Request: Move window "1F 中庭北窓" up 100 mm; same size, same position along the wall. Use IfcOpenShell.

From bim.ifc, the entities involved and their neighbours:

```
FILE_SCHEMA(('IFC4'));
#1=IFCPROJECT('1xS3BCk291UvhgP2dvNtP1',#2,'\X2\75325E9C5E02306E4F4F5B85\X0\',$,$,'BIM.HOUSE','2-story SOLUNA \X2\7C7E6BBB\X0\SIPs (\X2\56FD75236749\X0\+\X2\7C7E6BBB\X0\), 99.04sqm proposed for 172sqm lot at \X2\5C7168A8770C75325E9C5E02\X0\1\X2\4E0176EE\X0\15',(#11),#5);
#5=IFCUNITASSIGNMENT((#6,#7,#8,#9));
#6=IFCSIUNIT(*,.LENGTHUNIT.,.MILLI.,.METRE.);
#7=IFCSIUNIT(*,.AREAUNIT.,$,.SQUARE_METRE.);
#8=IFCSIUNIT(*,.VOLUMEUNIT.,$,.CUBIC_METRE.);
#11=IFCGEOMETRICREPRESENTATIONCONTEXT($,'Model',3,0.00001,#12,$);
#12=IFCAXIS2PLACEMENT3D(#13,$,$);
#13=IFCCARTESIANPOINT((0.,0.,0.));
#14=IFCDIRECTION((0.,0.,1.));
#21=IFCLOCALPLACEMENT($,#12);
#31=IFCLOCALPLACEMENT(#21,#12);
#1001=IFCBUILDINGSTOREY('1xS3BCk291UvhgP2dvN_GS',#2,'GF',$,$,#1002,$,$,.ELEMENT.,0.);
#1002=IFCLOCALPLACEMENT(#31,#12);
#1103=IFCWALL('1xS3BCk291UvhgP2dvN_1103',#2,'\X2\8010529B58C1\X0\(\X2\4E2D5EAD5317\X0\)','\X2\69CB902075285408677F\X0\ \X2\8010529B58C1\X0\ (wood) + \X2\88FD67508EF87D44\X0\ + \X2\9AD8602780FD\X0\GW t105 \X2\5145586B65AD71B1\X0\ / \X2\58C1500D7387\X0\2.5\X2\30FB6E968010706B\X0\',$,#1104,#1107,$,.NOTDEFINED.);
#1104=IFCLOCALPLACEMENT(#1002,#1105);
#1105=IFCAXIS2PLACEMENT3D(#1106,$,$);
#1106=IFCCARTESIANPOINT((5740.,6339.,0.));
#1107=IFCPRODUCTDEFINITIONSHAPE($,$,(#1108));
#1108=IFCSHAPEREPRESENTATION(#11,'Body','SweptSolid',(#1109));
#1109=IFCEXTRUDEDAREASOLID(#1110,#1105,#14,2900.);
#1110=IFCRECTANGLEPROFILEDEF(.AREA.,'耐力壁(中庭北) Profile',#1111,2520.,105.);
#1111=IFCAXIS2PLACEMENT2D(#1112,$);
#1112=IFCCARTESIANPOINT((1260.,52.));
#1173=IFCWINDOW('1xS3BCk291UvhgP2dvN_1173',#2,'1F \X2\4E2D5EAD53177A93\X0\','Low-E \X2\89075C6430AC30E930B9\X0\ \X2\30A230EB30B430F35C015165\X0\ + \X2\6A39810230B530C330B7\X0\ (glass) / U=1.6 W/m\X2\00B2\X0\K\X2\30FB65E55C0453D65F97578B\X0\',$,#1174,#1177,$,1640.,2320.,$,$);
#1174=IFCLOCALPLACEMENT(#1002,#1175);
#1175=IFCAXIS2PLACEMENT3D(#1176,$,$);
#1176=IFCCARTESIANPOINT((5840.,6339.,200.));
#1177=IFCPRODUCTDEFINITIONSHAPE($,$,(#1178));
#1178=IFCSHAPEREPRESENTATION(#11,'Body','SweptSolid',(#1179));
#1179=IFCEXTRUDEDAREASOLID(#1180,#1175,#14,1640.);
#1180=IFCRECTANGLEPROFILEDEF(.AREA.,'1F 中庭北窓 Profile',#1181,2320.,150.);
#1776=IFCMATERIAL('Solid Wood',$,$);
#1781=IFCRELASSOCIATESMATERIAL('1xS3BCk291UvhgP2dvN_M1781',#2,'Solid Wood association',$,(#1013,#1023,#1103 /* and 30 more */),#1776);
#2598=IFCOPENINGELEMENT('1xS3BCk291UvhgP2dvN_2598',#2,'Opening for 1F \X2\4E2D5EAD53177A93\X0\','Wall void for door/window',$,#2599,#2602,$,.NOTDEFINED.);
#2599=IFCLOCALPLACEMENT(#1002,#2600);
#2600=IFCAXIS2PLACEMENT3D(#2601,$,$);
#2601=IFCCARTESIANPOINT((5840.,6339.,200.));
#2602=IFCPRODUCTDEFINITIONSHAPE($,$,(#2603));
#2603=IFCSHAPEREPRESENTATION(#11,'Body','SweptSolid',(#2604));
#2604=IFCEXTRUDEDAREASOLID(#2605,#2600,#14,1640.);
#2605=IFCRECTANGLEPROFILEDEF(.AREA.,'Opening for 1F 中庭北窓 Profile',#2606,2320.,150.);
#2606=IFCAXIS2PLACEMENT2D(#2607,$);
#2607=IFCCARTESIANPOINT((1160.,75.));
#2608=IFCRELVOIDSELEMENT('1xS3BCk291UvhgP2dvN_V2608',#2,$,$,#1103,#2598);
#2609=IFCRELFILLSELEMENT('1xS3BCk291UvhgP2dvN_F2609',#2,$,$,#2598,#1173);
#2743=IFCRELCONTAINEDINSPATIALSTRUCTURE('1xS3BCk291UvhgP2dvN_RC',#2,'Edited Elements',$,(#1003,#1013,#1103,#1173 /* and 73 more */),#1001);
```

```python
import numpy as np
import ifcopenshell
import ifcopenshell.api.geometry
import ifcopenshell.util.placement
import ifcopenshell.util.unit

model = ifcopenshell.open("bim.ifc")
unit_scale = ifcopenshell.util.unit.calculate_unit_scale(model)

window = model.by_guid("1xS3BCk291UvhgP2dvN_1173")
opening = window.FillsVoids[0].RelatingOpeningElement
dz = 0.1 / unit_scale

shift = np.array([0.0, 0.0, dz])
# The window is not placed relative to its opening, so move both.
for product in (opening, window):
    matrix = ifcopenshell.util.placement.get_local_placement(product.ObjectPlacement)
    matrix[:3, 3] += shift
    ifcopenshell.api.geometry.edit_object_placement(model, product=product, matrix=matrix, is_si=False)

print(f"moved by {dz * unit_scale:+.3f} m")

model.write("bim_edited.ifc")
```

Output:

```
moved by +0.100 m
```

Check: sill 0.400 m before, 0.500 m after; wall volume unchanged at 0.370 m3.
